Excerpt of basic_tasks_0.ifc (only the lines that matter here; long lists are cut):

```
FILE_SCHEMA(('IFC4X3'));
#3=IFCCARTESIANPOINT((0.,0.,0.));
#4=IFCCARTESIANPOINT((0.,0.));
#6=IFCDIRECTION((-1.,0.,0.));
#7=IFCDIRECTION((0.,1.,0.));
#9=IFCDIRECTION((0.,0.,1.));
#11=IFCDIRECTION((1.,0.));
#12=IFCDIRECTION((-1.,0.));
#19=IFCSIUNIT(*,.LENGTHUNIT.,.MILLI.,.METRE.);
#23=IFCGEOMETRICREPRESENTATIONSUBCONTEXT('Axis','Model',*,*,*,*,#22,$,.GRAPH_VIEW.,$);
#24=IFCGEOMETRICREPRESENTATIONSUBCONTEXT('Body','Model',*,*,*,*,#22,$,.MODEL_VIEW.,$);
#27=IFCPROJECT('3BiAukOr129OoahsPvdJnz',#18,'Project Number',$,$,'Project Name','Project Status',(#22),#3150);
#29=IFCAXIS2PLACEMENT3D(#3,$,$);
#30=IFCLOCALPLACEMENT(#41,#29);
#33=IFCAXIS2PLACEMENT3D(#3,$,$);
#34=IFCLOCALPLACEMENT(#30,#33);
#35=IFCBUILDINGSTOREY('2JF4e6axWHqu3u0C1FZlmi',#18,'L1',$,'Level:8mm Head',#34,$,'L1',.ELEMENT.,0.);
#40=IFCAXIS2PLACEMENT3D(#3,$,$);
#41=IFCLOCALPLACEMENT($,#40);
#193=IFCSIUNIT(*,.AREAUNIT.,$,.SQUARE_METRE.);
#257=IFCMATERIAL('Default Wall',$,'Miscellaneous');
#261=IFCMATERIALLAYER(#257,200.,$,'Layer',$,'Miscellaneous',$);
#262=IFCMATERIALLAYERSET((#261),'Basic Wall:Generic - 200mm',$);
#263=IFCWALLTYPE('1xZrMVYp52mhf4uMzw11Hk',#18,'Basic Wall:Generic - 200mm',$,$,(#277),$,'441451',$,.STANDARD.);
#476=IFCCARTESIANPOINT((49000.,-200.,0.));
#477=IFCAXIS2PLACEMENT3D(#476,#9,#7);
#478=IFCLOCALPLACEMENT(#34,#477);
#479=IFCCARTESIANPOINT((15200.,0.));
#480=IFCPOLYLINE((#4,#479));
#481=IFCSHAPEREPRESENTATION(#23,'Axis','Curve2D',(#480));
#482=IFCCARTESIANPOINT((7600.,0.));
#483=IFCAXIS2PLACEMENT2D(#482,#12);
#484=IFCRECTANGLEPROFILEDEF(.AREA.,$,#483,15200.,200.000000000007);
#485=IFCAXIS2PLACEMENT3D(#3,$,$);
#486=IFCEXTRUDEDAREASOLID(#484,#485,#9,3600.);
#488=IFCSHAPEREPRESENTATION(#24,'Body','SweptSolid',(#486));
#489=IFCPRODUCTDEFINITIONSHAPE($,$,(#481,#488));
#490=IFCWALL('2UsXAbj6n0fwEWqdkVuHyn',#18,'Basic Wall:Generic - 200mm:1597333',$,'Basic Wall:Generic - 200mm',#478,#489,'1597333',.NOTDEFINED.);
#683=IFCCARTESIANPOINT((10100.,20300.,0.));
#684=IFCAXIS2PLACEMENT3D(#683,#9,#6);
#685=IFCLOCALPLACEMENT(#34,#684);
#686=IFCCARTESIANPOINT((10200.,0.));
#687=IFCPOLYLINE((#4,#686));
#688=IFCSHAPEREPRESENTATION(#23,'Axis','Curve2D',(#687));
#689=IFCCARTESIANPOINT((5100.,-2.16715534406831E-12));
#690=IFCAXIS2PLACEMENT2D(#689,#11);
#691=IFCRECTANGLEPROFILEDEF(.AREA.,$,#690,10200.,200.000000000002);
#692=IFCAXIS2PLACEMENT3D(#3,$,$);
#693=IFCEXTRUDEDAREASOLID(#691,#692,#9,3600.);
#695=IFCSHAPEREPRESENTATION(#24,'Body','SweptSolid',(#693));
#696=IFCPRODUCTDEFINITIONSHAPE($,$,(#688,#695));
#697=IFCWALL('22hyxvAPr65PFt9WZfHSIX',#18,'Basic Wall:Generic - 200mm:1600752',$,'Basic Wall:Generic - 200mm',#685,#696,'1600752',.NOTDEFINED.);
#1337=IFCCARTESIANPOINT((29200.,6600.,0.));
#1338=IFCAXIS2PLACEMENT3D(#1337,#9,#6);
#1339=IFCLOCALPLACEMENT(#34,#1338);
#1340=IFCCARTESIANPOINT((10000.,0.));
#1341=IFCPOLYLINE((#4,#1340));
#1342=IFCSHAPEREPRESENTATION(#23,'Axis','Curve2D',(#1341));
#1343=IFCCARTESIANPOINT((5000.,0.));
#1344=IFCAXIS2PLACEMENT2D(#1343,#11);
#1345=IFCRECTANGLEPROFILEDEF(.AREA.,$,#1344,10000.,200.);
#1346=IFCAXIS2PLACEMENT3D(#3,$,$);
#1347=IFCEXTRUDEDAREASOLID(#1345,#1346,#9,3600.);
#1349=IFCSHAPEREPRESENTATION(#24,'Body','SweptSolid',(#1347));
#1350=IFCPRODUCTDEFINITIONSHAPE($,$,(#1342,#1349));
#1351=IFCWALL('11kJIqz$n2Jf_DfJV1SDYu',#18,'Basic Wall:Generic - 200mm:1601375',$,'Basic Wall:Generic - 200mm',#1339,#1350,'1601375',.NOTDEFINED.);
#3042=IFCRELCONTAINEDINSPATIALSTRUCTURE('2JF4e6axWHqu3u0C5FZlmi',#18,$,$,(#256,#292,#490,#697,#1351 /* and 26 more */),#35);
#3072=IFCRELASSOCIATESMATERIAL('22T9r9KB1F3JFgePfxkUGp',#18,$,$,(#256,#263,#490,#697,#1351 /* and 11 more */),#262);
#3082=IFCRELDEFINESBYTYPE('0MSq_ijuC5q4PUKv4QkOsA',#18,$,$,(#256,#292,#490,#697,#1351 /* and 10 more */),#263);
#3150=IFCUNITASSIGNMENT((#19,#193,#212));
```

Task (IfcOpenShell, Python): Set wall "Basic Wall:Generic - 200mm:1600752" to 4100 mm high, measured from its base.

```python
import ifcopenshell
import ifcopenshell.geom
import ifcopenshell.util.representation
import ifcopenshell.util.shape

model = ifcopenshell.open("basic_tasks_0.ifc")
settings = ifcopenshell.geom.settings()


def volume(element):
    """Net volume in cubic metres, openings subtracted."""
    shape = ifcopenshell.geom.create_shape(settings, element)
    return ifcopenshell.util.shape.get_volume(shape.geometry)


wall = model.by_guid("22hyxvAPr65PFt9WZfHSIX")
before = volume(wall)

body = ifcopenshell.util.representation.get_representation(wall, "Model", "Body")
solid = body.Items[0]
old_height = solid.Depth
solid.Depth = 4100.0
after = volume(wall)

print(f"height {old_height:g} -> {solid.Depth:g}, volume {before:.3f} -> {after:.3f} m3")

model.write("basic_tasks_0_rev.ifc")
```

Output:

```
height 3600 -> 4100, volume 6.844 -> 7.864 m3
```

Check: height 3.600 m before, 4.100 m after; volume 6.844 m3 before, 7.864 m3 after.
